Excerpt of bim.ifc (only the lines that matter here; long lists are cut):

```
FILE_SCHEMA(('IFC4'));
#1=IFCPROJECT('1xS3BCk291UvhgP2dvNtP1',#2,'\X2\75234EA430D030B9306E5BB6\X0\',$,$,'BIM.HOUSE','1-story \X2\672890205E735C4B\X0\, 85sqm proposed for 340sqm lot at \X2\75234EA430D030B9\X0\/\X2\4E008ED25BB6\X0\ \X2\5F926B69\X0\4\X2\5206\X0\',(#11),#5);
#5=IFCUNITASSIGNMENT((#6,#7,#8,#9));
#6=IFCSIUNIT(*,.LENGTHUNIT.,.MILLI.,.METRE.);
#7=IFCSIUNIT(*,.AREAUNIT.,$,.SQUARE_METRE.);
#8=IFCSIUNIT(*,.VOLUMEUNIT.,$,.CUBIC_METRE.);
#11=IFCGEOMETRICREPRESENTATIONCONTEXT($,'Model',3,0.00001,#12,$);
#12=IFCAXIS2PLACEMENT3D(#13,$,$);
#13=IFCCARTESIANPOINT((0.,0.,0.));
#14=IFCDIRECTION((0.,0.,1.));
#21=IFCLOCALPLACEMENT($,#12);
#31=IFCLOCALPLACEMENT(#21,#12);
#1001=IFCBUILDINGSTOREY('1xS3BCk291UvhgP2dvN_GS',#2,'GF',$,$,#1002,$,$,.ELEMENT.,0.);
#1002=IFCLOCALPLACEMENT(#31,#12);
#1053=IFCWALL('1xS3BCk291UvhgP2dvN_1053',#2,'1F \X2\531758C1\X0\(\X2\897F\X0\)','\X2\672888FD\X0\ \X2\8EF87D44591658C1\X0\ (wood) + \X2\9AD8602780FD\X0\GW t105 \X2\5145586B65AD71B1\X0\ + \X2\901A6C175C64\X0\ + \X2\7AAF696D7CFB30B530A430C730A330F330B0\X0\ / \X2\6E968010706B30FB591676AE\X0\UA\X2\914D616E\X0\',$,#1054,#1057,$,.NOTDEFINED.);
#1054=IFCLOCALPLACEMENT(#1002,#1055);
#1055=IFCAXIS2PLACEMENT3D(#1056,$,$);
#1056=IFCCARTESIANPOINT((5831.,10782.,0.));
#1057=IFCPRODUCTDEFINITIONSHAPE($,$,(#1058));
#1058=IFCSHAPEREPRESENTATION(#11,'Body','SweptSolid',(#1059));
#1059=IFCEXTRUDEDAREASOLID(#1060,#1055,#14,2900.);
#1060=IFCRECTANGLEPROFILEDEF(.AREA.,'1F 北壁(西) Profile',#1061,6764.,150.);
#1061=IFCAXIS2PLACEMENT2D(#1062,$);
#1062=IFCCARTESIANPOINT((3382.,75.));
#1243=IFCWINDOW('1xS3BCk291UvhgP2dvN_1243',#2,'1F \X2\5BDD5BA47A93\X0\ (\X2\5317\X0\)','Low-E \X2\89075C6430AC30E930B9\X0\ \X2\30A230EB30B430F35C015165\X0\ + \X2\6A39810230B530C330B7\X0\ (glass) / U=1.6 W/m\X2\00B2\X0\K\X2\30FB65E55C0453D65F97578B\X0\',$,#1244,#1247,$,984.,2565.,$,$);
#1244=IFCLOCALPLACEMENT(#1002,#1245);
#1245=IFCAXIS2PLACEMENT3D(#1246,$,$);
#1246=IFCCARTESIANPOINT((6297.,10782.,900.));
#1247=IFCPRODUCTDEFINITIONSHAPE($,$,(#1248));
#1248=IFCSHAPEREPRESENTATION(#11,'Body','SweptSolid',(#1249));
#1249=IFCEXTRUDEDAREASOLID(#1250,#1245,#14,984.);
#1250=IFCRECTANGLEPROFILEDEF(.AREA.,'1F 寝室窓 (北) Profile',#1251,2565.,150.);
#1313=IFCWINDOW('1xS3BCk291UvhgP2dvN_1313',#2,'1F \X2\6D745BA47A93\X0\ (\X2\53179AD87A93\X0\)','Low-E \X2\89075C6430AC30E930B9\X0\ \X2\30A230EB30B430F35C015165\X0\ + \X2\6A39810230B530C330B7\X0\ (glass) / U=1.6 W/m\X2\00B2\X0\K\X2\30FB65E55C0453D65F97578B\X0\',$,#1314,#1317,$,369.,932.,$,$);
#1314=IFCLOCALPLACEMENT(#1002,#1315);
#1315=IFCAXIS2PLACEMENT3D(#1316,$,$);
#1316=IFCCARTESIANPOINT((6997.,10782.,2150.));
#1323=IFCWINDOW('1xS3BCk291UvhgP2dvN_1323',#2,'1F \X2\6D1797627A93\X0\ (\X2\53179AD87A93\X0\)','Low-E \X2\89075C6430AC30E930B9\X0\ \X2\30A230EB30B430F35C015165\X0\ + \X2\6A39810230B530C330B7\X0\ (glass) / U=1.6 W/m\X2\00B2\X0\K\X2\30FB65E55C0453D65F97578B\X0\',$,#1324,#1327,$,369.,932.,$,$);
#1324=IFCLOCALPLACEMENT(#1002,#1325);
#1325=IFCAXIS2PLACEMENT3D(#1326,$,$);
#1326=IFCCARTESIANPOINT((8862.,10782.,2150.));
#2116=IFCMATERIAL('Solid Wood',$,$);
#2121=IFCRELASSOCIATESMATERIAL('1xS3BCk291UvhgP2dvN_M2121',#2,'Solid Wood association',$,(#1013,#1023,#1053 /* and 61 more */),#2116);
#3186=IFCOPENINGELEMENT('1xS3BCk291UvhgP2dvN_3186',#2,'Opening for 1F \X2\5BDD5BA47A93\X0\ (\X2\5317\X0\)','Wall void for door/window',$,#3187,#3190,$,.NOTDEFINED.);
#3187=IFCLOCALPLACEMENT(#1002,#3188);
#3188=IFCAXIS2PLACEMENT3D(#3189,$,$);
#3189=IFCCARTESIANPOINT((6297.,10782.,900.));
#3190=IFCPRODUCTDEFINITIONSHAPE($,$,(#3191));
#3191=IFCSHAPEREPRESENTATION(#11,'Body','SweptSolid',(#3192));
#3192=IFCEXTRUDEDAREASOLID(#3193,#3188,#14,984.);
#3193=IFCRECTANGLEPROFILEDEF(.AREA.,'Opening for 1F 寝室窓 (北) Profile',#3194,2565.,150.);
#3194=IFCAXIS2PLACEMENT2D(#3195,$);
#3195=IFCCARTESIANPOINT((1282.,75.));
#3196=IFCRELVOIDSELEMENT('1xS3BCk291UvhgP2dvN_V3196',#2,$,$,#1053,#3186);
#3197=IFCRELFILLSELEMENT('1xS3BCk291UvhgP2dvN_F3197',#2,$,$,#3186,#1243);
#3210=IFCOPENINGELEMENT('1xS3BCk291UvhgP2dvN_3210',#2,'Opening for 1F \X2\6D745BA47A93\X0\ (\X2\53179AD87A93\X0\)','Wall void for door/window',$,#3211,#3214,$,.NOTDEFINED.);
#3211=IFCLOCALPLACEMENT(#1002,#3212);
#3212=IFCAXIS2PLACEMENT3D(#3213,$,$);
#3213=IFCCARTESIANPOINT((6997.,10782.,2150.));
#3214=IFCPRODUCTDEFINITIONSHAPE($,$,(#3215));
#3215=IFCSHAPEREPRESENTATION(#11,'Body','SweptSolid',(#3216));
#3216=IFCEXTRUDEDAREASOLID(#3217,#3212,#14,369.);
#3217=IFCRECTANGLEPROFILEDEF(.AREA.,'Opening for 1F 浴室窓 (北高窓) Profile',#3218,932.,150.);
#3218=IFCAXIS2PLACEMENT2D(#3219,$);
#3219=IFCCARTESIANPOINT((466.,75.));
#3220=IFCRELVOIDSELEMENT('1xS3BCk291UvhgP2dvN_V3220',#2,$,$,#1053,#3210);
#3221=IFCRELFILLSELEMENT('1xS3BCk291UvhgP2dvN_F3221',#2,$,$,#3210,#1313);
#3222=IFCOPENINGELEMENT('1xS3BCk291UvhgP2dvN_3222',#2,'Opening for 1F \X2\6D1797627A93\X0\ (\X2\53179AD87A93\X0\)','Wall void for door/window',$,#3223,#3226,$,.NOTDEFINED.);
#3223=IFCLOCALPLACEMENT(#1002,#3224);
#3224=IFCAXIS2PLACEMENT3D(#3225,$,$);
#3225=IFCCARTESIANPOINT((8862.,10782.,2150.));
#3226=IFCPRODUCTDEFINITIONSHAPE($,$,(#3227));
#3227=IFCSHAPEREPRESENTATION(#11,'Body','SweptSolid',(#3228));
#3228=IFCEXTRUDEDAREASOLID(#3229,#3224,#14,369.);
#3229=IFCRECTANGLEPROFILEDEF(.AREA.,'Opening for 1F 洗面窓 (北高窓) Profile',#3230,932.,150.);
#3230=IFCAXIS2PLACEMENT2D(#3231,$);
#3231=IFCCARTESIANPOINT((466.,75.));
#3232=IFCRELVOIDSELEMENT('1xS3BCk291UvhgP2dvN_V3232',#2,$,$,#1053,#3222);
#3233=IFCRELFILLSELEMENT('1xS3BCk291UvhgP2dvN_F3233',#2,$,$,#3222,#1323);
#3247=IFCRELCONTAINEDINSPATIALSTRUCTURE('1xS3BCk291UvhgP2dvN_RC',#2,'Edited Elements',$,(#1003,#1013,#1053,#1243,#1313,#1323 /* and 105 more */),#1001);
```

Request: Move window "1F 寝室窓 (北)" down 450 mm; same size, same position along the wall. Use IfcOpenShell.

```python
import numpy as np
import ifcopenshell
import ifcopenshell.api.geometry
import ifcopenshell.util.placement
import ifcopenshell.util.unit

model = ifcopenshell.open("bim.ifc")
unit_scale = ifcopenshell.util.unit.calculate_unit_scale(model)

window = model.by_guid("1xS3BCk291UvhgP2dvN_1243")
opening = window.FillsVoids[0].RelatingOpeningElement
dz = -0.45 / unit_scale

shift = np.array([0.0, 0.0, dz])
# The window is not placed relative to its opening, so move both.
for product in (opening, window):
    matrix = ifcopenshell.util.placement.get_local_placement(product.ObjectPlacement)
    matrix[:3, 3] += shift
    ifcopenshell.api.geometry.edit_object_placement(model, product=product, matrix=matrix, is_si=False)

print(f"moved by {dz * unit_scale:+.3f} m")

model.write("bim_updated.ifc")
```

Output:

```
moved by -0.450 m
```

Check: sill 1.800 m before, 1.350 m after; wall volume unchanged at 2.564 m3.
